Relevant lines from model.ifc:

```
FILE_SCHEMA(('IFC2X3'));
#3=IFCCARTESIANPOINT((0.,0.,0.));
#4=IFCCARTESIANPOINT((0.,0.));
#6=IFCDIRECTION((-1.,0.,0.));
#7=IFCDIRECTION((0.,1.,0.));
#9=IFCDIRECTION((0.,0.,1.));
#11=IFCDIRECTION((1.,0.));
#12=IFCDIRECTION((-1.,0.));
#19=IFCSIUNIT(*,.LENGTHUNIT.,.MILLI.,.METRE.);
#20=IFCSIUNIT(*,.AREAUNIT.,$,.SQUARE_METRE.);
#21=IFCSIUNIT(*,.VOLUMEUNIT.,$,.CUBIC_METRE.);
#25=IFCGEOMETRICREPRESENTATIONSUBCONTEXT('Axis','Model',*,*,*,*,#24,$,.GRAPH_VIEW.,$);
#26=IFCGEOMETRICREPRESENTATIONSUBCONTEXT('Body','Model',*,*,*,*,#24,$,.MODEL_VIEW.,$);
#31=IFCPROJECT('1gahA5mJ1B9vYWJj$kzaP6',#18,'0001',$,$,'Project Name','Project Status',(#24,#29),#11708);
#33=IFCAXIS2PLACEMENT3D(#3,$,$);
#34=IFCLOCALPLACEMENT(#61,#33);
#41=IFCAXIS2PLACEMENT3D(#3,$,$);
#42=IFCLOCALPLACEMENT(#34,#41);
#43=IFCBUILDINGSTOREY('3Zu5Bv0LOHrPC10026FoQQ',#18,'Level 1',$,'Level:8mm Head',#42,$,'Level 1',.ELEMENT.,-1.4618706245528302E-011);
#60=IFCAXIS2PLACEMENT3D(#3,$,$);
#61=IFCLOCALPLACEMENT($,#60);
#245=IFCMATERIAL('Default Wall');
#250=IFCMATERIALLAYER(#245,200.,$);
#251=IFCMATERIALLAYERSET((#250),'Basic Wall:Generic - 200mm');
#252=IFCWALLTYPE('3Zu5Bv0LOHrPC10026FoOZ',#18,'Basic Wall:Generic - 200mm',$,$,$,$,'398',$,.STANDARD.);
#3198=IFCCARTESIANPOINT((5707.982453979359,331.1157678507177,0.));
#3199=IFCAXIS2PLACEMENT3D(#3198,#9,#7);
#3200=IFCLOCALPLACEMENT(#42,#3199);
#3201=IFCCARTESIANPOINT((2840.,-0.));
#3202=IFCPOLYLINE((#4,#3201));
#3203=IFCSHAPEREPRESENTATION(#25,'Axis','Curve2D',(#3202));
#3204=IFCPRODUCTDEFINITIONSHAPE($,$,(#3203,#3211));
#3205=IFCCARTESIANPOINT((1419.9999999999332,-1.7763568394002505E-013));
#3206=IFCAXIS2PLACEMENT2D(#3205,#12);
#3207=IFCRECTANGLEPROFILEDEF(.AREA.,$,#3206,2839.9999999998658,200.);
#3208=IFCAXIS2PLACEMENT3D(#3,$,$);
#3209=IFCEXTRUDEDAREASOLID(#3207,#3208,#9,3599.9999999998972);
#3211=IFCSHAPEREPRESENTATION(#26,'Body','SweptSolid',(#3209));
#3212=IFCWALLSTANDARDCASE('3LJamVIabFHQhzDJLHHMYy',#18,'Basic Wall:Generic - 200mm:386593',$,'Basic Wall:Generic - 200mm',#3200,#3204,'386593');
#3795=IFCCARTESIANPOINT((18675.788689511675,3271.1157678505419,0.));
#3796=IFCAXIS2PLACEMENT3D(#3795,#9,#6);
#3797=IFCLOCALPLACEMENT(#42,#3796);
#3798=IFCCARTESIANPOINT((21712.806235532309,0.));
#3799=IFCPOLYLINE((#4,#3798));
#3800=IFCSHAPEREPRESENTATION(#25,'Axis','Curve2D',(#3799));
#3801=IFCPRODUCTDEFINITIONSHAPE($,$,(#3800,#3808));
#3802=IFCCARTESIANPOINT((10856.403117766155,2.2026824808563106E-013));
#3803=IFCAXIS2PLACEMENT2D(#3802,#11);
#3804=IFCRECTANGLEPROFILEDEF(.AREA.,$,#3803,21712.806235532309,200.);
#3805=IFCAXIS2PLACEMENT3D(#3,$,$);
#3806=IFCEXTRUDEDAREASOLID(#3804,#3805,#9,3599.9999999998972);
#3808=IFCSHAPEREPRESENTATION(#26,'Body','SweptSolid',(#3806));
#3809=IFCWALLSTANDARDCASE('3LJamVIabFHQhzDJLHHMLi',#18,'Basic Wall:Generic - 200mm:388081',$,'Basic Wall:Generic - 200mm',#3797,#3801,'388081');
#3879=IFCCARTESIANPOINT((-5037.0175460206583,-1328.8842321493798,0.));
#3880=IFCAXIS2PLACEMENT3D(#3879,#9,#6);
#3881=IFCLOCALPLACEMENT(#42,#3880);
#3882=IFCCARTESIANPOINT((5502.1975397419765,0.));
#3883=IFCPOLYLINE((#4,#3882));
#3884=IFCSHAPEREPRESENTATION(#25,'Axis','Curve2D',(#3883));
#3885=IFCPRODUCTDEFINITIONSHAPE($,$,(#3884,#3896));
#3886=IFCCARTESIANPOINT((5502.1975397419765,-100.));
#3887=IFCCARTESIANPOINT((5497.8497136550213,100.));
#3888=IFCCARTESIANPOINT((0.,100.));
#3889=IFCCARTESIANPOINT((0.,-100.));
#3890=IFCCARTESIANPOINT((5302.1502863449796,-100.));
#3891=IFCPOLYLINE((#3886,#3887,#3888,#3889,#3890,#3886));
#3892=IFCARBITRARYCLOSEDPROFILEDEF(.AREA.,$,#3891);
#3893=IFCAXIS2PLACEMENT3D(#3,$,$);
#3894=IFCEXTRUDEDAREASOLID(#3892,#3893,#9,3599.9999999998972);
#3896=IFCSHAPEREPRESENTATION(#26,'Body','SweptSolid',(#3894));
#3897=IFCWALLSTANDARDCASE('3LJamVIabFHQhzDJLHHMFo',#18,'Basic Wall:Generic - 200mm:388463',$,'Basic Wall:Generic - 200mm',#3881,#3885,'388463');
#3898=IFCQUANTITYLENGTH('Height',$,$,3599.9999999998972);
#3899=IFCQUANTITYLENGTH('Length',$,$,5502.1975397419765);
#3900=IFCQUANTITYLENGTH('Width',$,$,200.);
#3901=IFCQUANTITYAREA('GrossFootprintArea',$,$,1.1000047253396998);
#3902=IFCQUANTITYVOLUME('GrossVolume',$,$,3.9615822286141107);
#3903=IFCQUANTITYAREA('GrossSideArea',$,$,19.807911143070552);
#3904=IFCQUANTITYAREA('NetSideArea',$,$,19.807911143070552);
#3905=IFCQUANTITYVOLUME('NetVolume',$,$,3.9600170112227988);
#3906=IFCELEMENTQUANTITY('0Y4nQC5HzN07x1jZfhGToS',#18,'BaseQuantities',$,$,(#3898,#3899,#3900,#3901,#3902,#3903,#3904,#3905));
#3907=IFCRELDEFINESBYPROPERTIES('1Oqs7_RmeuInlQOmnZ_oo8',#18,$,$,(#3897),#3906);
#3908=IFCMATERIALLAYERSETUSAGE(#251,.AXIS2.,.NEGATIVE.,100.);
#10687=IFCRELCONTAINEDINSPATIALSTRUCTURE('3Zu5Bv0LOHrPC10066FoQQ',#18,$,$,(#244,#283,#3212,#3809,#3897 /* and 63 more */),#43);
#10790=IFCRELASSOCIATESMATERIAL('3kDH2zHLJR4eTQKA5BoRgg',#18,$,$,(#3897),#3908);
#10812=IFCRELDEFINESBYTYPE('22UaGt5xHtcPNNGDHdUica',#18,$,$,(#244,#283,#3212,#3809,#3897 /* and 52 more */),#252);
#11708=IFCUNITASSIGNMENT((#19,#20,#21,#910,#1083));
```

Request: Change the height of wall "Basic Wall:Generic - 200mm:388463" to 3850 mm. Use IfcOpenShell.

```python
import ifcopenshell
import ifcopenshell.api.pset
import ifcopenshell.geom
import ifcopenshell.util.element
import ifcopenshell.util.representation
import ifcopenshell.util.shape
import ifcopenshell.util.unit

model = ifcopenshell.open("model.ifc")
unit_scale = ifcopenshell.util.unit.calculate_unit_scale(model)
area_scale = ifcopenshell.util.unit.calculate_unit_scale(model, "AREAUNIT")
volume_scale = ifcopenshell.util.unit.calculate_unit_scale(model, "VOLUMEUNIT")
settings = ifcopenshell.geom.settings()


def volume(element):
    """Net volume in cubic metres, openings subtracted."""
    shape = ifcopenshell.geom.create_shape(settings, element)
    return ifcopenshell.util.shape.get_volume(shape.geometry)


wall = model.by_guid("3LJamVIabFHQhzDJLHHMFo")
before = volume(wall)

body = ifcopenshell.util.representation.get_representation(wall, "Model", "Body")
solid = body.Items[0]
old_height = solid.Depth
solid.Depth = 3.85 / unit_scale
after = volume(wall)
thickness = 0.2  # wall thickness in metres

# Update the stored height, areas and volumes.
qto = model.by_id(ifcopenshell.util.element.get_pset(wall, "BaseQuantities", should_inherit=False)["id"])
ifcopenshell.api.pset.edit_qto(model, qto=qto, properties={
    "Height": solid.Depth,
    "GrossVolume": ifcopenshell.util.element.get_pset(wall, "BaseQuantities", "GrossVolume") * solid.Depth / old_height,
    "GrossSideArea": ifcopenshell.util.element.get_pset(wall, "BaseQuantities", "GrossSideArea") * solid.Depth / old_height,
    "NetSideArea": after / thickness / area_scale,
    "NetVolume": after / volume_scale,
})

print(f"height {old_height:g} -> {solid.Depth:g}, volume {before:.3f} -> {after:.3f} m3")

model.write("model_updated.ifc")
```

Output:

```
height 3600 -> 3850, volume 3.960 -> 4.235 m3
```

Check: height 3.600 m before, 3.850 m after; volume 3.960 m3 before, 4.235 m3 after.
